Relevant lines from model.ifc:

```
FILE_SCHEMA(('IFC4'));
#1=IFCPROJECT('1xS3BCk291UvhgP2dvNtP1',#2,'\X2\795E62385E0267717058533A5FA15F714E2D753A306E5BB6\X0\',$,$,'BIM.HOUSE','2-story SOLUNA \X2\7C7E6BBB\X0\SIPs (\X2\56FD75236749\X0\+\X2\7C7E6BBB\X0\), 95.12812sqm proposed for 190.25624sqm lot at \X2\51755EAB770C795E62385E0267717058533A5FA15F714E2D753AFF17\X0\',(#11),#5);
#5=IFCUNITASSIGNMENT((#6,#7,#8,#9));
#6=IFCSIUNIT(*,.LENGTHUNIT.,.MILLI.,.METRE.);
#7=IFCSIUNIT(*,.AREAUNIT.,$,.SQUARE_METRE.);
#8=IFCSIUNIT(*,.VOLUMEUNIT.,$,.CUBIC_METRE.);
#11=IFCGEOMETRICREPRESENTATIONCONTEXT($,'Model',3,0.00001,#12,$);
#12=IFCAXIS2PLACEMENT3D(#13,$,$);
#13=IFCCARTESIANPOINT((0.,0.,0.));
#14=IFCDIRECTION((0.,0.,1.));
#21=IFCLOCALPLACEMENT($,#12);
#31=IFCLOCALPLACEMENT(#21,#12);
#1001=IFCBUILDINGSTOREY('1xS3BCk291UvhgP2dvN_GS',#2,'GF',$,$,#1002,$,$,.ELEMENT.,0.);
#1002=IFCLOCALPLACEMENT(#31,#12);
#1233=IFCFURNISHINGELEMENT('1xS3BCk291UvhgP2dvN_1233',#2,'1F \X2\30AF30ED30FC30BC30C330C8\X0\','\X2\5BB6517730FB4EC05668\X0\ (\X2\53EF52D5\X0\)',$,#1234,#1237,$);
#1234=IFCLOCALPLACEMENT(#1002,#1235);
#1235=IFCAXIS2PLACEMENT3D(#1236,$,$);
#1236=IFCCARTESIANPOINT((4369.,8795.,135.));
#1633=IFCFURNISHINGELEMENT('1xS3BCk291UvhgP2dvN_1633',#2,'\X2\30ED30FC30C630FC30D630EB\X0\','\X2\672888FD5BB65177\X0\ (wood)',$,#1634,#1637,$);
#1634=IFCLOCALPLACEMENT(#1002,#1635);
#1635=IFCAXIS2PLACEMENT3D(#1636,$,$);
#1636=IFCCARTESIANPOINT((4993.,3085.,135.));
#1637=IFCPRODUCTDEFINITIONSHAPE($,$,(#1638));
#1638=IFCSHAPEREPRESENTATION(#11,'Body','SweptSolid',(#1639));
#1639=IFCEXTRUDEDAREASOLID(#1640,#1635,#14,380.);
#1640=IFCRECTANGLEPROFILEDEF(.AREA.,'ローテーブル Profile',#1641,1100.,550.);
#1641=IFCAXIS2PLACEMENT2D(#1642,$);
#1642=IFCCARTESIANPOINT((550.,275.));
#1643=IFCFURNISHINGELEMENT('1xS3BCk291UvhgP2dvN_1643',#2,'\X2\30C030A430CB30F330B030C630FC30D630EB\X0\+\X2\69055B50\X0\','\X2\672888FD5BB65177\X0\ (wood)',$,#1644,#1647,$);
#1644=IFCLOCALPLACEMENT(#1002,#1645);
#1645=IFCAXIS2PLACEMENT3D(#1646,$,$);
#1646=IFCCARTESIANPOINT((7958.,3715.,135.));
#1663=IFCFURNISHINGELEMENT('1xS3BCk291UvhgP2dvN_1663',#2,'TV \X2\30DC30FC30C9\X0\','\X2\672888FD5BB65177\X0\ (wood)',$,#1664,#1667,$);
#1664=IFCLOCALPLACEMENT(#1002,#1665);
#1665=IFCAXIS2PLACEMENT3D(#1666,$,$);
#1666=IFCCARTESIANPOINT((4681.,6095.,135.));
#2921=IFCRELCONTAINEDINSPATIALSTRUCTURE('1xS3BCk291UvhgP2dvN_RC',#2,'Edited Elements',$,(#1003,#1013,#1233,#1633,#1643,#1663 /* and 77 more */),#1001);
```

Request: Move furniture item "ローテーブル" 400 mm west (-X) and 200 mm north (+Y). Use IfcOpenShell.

```python
import ifcopenshell
import ifcopenshell.api.geometry
import ifcopenshell.util.placement

model = ifcopenshell.open("model.ifc")

item = model.by_guid("1xS3BCk291UvhgP2dvN_1633")
matrix = ifcopenshell.util.placement.get_local_placement(item.ObjectPlacement)
matrix[0, 3] -= 400.0
matrix[1, 3] += 200.0
ifcopenshell.api.geometry.edit_object_placement(model, product=item, matrix=matrix, is_si=False)

print(ifcopenshell.util.placement.get_local_placement(item.ObjectPlacement).round(3) + 0.0)

model.write("model_rev.ifc")
```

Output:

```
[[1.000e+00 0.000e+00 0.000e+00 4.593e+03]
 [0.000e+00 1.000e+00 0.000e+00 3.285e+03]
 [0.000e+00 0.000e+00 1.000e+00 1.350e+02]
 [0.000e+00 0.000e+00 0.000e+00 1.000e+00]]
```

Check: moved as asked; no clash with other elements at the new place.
